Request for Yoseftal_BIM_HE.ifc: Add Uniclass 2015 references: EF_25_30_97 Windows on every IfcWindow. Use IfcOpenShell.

First a look at what the model holds.

```python
import ifcopenshell

model = ifcopenshell.open("Yoseftal_BIM_HE.ifc")
print(model.schema)
print("classifications:", [c.Name for c in model.by_type("IfcClassification")])
for ifc_class in ("IfcDoor", "IfcRoof", "IfcStair", "IfcWall", "IfcWindow"):
    print(ifc_class, len(model.by_type(ifc_class)))
```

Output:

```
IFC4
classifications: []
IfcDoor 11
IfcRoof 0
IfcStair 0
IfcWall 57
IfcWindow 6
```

```python
import ifcopenshell
import ifcopenshell.api.classification

model = ifcopenshell.open("Yoseftal_BIM_HE.ifc")

system = ifcopenshell.api.classification.add_classification(model, classification="Uniclass 2015")

codes = {
    "IfcWindow": ("EF_25_30_97", "Windows"),
}
for ifc_class, (code, name) in codes.items():
    products = model.by_type(ifc_class)
    ifcopenshell.api.classification.add_reference(
        model, products=products, classification=system, identification=code, name=name
    )
    print(code, len(products))

model.write("Yoseftal_BIM_HE_v2.ifc")
```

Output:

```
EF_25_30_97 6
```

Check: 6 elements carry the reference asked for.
